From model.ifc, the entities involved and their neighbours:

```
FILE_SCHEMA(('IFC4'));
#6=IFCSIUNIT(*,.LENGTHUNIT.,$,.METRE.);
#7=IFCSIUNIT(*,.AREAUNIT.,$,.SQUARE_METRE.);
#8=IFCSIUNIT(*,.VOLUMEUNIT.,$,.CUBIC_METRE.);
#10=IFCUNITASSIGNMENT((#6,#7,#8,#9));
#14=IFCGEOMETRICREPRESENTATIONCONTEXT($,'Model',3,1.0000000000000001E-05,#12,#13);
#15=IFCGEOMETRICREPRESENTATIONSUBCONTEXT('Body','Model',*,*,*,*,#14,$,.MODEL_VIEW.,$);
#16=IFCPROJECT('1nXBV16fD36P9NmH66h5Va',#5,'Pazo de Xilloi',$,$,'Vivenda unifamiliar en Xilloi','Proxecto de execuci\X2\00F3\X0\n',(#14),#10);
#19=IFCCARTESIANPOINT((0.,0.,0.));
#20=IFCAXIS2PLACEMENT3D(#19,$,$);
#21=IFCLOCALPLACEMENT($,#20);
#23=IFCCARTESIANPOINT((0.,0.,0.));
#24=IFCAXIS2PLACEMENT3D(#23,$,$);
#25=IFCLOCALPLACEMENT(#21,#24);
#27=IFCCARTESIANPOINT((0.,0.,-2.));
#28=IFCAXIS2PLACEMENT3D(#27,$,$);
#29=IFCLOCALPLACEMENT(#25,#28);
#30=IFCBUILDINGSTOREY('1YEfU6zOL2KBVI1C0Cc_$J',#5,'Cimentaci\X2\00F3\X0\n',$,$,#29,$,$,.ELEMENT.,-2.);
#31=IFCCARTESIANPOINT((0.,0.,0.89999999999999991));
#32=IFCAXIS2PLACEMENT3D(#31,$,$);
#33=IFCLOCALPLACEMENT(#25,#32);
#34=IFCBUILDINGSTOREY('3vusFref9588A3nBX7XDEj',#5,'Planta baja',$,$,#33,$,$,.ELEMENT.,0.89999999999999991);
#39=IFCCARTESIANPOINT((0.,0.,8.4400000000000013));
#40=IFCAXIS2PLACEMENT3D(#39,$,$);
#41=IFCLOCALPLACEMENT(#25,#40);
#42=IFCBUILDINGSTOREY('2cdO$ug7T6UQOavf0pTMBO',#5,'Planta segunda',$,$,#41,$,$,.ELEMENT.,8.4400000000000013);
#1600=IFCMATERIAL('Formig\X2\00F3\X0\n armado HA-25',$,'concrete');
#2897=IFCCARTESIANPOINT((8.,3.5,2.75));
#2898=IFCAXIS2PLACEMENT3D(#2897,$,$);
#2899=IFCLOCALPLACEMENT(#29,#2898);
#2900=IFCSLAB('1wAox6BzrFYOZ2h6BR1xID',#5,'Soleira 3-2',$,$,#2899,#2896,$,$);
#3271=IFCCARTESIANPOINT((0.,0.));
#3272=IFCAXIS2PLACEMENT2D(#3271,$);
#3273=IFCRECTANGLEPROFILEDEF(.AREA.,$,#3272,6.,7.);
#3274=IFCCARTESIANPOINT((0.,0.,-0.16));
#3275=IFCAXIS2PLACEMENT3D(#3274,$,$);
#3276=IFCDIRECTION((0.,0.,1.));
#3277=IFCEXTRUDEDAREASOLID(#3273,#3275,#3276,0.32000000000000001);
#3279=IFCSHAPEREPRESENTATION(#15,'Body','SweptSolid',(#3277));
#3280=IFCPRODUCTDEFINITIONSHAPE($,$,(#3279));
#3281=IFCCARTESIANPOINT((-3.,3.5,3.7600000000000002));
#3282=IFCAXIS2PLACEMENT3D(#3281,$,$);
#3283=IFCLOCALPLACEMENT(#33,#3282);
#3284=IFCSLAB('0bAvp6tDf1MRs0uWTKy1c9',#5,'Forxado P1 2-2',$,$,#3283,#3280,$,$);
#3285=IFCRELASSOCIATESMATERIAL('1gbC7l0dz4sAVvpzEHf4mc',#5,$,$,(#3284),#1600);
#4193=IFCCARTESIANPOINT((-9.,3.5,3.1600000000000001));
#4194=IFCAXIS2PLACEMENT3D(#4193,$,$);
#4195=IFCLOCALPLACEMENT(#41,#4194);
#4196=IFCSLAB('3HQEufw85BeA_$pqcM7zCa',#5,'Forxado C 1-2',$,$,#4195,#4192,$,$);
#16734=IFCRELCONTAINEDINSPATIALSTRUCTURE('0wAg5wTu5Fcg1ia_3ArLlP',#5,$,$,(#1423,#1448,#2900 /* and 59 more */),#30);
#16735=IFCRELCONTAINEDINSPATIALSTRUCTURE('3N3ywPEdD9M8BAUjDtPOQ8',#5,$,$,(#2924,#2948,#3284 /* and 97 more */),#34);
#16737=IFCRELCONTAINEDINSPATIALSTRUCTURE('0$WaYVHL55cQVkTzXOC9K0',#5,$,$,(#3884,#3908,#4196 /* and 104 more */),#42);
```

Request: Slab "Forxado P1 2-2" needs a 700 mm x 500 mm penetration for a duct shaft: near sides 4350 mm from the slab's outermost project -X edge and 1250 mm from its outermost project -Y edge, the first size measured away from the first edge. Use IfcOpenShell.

```python
import numpy as np
import ifcopenshell
import ifcopenshell.api.feature
import ifcopenshell.api.geometry
import ifcopenshell.api.root
import ifcopenshell.geom
import ifcopenshell.util.placement
import ifcopenshell.util.representation
import ifcopenshell.util.shape
import ifcopenshell.util.unit

model = ifcopenshell.open("model.ifc")
unit_scale = ifcopenshell.util.unit.calculate_unit_scale(model)
settings = ifcopenshell.geom.settings()


def volume(element):
    """Net volume in cubic metres, openings subtracted."""
    shape = ifcopenshell.geom.create_shape(settings, element)
    return ifcopenshell.util.shape.get_volume(shape.geometry)


slab = model.by_guid("0bAvp6tDf1MRs0uWTKy1c9")
before = volume(slab)

# Extent in the slab's own axes, in metres. The edges named are its -X and -Y sides.
slab_shape = ifcopenshell.geom.create_shape(settings, slab)
vertices = ifcopenshell.util.shape.get_vertices(slab_shape.geometry)
x_min, y_min, bottom = vertices.min(axis=0)
top = vertices[:, 2].max()

opening = ifcopenshell.api.root.create_entity(model, ifc_class="IfcOpeningElement", name="Duct shaft opening", predefined_type="OPENING")
context = ifcopenshell.util.representation.get_context(model, "Model", "Body", "MODEL_VIEW")
width, depth = 0.7, 0.5
outline = [(0.0, 0.0), (width, 0.0), (width, depth), (0.0, depth), (0.0, 0.0)]
# Overshoot both faces by 50 mm so the cut is clean.
shape = ifcopenshell.api.geometry.add_slab_representation(
    model, context=context, depth=top - bottom + 0.1, polyline=outline
)
ifcopenshell.api.geometry.assign_representation(model, product=opening, representation=shape)

matrix = ifcopenshell.util.placement.get_local_placement(slab.ObjectPlacement)
matrix[:, 3] = matrix @ np.append(np.array([x_min + 4.35, y_min + 1.25, bottom - 0.05]) / unit_scale, 1.0)
ifcopenshell.api.geometry.edit_object_placement(model, product=opening, matrix=matrix, is_si=False)
ifcopenshell.api.feature.add_feature(model, feature=opening, element=slab)

after = volume(slab)

print(f"slab volume {before:.3f} -> {after:.3f} m3")

model.write("model_rev.ifc")
```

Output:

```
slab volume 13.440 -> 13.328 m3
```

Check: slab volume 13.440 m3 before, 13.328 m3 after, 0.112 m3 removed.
